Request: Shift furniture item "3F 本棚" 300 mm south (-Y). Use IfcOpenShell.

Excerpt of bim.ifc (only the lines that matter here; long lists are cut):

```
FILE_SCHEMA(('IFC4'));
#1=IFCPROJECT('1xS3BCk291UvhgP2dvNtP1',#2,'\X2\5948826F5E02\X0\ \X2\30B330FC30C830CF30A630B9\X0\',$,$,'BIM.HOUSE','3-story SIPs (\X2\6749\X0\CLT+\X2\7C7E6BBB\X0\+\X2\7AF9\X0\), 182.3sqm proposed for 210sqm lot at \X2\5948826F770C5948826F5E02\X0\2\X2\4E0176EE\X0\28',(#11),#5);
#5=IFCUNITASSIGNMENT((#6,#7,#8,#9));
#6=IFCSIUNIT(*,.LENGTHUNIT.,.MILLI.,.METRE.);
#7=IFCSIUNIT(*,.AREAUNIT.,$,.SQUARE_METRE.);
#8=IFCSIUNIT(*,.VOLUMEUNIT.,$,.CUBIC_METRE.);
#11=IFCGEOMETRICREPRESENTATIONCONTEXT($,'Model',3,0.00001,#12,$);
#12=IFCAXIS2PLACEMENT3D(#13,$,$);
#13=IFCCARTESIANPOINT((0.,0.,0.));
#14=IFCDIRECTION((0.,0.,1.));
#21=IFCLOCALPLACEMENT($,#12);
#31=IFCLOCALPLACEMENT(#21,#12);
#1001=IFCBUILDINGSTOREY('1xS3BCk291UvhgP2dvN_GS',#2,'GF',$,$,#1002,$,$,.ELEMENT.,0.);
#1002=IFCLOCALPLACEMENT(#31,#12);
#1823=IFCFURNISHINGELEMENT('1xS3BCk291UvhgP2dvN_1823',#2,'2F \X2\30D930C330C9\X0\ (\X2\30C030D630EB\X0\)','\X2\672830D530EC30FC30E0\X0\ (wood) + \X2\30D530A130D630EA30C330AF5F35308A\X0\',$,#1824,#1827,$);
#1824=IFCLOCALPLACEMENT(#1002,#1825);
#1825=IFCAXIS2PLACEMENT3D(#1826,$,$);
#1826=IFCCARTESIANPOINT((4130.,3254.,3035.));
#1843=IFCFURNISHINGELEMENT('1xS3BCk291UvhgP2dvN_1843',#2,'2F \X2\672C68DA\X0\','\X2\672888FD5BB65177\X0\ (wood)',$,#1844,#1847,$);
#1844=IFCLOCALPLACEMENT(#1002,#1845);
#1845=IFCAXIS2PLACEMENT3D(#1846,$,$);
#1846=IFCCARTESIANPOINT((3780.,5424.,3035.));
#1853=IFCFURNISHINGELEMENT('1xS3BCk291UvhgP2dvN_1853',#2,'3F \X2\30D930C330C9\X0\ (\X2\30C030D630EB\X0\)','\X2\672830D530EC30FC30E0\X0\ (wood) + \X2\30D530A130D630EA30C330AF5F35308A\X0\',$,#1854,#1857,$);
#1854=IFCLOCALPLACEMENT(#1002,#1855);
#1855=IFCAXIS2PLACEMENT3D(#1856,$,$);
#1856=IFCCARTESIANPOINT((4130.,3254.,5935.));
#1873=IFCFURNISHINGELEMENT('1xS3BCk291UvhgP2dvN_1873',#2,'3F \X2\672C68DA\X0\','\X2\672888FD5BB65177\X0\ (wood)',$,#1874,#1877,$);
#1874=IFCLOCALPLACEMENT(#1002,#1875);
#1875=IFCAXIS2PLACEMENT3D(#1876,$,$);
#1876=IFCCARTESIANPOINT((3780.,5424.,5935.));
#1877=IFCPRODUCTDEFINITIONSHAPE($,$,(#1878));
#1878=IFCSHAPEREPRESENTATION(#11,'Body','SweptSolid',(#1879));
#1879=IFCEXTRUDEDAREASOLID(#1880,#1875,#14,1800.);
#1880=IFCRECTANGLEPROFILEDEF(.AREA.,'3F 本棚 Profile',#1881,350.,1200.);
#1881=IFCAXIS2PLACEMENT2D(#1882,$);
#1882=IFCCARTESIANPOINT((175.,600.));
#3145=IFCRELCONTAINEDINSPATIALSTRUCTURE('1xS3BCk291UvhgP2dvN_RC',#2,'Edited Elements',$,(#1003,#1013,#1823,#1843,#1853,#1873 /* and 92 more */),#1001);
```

```python
import ifcopenshell
import ifcopenshell.api.geometry
import ifcopenshell.util.placement
import ifcopenshell.util.unit

model = ifcopenshell.open("bim.ifc")
unit_scale = ifcopenshell.util.unit.calculate_unit_scale(model)

item = model.by_guid("1xS3BCk291UvhgP2dvN_1873")
matrix = ifcopenshell.util.placement.get_local_placement(item.ObjectPlacement)
matrix[1, 3] -= 0.3 / unit_scale
ifcopenshell.api.geometry.edit_object_placement(model, product=item, matrix=matrix, is_si=False)

print(ifcopenshell.util.placement.get_local_placement(item.ObjectPlacement).round(3) + 0.0)

model.write("bim_v2.ifc")
```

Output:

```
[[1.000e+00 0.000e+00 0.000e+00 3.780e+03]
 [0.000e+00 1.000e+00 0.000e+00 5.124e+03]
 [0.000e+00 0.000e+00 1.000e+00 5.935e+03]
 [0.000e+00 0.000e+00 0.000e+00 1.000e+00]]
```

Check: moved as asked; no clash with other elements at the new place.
